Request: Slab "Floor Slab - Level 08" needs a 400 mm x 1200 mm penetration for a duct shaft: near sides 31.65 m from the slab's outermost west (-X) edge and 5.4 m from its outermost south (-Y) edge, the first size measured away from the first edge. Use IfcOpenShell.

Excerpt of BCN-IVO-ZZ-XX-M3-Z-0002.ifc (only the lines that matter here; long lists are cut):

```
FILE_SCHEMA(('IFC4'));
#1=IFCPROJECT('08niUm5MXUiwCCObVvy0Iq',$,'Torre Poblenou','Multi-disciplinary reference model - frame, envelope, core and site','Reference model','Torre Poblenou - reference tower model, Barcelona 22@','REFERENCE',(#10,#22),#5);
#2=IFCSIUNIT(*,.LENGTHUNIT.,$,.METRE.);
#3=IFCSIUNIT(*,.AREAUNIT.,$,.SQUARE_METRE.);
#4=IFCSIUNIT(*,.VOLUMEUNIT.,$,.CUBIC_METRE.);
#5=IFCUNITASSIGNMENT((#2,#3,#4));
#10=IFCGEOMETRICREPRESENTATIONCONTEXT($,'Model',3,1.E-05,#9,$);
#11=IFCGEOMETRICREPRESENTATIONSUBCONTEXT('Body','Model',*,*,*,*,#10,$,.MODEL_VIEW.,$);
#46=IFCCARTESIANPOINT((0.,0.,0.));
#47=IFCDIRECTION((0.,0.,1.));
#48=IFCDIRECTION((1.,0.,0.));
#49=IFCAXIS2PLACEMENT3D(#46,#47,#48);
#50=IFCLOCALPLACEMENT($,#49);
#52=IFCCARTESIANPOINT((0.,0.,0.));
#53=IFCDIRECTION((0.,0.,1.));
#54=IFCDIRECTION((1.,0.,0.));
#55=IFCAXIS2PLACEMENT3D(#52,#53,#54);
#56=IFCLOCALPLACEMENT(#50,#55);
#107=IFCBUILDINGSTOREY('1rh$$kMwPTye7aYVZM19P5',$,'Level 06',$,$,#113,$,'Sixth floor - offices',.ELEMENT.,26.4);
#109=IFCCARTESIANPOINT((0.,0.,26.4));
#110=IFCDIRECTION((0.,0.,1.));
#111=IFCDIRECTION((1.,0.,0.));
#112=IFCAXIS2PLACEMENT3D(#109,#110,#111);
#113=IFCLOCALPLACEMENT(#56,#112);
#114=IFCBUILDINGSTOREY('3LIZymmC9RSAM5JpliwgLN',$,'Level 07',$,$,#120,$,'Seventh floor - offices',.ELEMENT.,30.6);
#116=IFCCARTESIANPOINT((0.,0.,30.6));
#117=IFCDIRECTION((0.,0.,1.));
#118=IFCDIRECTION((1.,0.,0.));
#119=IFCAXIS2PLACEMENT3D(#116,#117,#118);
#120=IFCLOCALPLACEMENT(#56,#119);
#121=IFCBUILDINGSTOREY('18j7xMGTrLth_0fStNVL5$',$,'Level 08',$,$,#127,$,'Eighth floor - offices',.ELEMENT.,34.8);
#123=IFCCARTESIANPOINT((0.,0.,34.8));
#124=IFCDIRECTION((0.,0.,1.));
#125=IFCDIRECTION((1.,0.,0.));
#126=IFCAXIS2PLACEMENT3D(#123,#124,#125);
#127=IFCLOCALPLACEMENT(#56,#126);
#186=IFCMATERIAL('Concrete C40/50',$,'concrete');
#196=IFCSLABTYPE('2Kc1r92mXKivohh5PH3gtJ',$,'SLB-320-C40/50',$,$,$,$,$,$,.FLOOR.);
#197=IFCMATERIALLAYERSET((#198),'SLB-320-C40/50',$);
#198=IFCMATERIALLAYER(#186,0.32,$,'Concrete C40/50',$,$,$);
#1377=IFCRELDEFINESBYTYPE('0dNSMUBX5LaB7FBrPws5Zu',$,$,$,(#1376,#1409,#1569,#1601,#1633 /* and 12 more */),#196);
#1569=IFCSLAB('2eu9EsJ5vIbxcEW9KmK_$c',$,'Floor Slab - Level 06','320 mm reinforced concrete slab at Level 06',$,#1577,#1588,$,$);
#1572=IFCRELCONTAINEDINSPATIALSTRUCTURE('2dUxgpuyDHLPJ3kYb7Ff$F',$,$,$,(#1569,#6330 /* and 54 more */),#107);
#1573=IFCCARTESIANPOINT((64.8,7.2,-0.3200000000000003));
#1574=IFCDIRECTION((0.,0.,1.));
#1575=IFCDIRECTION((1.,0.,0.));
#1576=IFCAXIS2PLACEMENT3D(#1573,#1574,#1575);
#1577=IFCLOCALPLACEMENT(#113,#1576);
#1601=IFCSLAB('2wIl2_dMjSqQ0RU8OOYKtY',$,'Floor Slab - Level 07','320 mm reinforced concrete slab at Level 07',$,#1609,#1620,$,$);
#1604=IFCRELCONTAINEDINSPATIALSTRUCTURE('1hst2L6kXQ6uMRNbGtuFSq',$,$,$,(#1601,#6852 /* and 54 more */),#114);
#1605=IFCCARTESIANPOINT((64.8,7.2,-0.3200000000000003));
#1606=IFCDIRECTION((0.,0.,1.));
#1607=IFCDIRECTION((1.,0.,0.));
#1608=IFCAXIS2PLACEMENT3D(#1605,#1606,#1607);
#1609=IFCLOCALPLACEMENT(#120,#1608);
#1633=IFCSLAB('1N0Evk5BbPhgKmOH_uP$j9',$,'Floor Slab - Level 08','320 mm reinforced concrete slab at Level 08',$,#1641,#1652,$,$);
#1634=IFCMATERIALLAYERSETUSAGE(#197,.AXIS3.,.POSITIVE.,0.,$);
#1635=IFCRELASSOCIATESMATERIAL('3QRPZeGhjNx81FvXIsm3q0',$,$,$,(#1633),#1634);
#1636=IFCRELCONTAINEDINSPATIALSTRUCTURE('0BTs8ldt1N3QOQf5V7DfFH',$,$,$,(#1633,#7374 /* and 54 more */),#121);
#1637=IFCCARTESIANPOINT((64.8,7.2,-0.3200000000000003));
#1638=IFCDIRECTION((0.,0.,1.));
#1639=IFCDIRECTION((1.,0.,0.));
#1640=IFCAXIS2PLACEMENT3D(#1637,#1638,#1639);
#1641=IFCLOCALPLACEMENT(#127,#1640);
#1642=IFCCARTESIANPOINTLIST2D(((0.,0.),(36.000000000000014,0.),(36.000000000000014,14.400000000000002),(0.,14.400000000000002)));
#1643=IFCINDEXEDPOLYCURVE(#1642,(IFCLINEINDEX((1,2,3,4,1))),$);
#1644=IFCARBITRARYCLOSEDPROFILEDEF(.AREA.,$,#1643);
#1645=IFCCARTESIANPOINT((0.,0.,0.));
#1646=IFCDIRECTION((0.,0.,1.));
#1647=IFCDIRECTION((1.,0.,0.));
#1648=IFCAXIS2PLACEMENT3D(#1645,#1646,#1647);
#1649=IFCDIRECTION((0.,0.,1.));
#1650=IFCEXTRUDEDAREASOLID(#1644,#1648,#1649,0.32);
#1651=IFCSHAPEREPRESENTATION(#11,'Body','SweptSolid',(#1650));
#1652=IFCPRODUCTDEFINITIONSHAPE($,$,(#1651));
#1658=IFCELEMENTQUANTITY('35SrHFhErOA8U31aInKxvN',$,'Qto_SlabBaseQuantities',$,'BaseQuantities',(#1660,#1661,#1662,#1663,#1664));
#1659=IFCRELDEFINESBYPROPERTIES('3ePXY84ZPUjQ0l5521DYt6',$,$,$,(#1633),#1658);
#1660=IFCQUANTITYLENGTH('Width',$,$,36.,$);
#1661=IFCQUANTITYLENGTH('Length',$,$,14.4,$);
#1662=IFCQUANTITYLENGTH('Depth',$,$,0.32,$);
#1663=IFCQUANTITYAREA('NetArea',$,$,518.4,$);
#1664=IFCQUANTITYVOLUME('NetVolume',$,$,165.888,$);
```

```python
import numpy as np
import ifcopenshell
import ifcopenshell.api.feature
import ifcopenshell.api.geometry
import ifcopenshell.api.pset
import ifcopenshell.api.root
import ifcopenshell.geom
import ifcopenshell.util.element
import ifcopenshell.util.placement
import ifcopenshell.util.representation
import ifcopenshell.util.shape
import ifcopenshell.util.unit

model = ifcopenshell.open("BCN-IVO-ZZ-XX-M3-Z-0002.ifc")
unit_scale = ifcopenshell.util.unit.calculate_unit_scale(model)
area_scale = ifcopenshell.util.unit.calculate_unit_scale(model, "AREAUNIT")
volume_scale = ifcopenshell.util.unit.calculate_unit_scale(model, "VOLUMEUNIT")
settings = ifcopenshell.geom.settings()


def volume(element):
    """Net volume in cubic metres, openings subtracted."""
    shape = ifcopenshell.geom.create_shape(settings, element)
    return ifcopenshell.util.shape.get_volume(shape.geometry)


slab = model.by_guid("1N0Evk5BbPhgKmOH_uP$j9")
before = volume(slab)

# Extent in the slab's own axes, in metres. The edges named are its -X and -Y sides.
slab_shape = ifcopenshell.geom.create_shape(settings, slab)
vertices = ifcopenshell.util.shape.get_vertices(slab_shape.geometry)
x_min, y_min, bottom = vertices.min(axis=0)
top = vertices[:, 2].max()

opening = ifcopenshell.api.root.create_entity(model, ifc_class="IfcOpeningElement", name="Duct shaft opening", predefined_type="OPENING")
context = ifcopenshell.util.representation.get_context(model, "Model", "Body", "MODEL_VIEW")
width, depth = 0.4, 1.2
outline = [(0.0, 0.0), (width, 0.0), (width, depth), (0.0, depth), (0.0, 0.0)]
# Overshoot both faces by 50 mm so the cut is clean.
shape = ifcopenshell.api.geometry.add_slab_representation(
    model, context=context, depth=top - bottom + 0.1, polyline=outline
)
ifcopenshell.api.geometry.assign_representation(model, product=opening, representation=shape)

matrix = ifcopenshell.util.placement.get_local_placement(slab.ObjectPlacement)
matrix[:, 3] = matrix @ np.append(np.array([x_min + 31.65, y_min + 5.4, bottom - 0.05]) / unit_scale, 1.0)
ifcopenshell.api.geometry.edit_object_placement(model, product=opening, matrix=matrix, is_si=False)
ifcopenshell.api.feature.add_feature(model, feature=opening, element=slab)

after = volume(slab)

# Update the slab's stored quantities.
qto = model.by_id(ifcopenshell.util.element.get_pset(slab, "Qto_SlabBaseQuantities", should_inherit=False)["id"])
ifcopenshell.api.pset.edit_qto(model, qto=qto, properties={
    "NetArea": after / (top - bottom) / area_scale,
    "NetVolume": after / volume_scale,
})

print(f"slab volume {before:.3f} -> {after:.3f} m3")

model.write("BCN-IVO-ZZ-XX-M3-Z-0002_rev.ifc")
```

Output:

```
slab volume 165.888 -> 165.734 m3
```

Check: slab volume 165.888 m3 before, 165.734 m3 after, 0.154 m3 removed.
